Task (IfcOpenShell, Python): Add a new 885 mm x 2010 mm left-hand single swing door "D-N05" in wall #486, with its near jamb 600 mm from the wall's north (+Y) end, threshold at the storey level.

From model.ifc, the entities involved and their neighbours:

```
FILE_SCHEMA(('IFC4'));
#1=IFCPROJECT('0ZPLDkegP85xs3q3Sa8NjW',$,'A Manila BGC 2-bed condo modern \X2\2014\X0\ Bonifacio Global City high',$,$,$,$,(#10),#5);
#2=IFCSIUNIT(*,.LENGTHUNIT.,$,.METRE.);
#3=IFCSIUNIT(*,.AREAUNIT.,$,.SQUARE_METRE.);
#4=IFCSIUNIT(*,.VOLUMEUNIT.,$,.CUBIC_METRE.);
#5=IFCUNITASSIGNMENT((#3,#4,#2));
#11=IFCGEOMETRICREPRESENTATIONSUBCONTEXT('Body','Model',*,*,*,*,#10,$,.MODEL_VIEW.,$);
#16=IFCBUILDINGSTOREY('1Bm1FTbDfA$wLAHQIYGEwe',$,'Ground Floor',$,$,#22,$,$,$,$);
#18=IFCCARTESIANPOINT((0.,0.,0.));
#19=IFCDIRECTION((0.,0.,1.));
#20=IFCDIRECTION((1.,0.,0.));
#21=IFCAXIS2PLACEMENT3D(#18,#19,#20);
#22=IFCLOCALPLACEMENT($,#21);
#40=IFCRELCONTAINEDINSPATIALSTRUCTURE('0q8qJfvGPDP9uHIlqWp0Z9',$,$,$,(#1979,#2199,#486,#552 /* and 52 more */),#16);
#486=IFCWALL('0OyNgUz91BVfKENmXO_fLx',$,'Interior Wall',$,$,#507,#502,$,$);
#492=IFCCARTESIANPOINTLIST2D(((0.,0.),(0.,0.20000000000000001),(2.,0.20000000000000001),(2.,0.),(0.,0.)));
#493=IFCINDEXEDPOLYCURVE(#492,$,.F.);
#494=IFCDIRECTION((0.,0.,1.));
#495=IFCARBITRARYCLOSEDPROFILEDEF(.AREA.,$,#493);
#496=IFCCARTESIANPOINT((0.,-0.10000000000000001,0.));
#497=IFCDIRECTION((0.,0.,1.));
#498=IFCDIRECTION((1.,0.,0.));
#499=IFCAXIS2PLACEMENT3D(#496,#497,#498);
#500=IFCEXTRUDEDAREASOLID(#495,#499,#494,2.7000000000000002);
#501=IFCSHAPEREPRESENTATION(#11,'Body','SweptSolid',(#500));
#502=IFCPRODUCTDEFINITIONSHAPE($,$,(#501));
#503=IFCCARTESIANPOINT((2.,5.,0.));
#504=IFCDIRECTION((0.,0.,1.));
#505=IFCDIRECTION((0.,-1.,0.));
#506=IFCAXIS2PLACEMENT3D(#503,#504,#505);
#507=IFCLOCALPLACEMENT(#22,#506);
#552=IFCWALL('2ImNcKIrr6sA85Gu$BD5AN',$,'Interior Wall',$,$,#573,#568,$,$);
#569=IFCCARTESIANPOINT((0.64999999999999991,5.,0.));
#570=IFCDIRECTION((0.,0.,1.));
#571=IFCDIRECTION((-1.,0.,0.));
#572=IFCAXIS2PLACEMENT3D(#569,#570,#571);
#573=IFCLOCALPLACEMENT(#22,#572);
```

```python
import numpy as np
import ifcopenshell
import ifcopenshell.api.feature
import ifcopenshell.api.geometry
import ifcopenshell.api.root
import ifcopenshell.api.spatial
import ifcopenshell.geom
import ifcopenshell.util.element
import ifcopenshell.util.placement
import ifcopenshell.util.representation
import ifcopenshell.util.shape
import ifcopenshell.util.unit

model = ifcopenshell.open("model.ifc")
unit_scale = ifcopenshell.util.unit.calculate_unit_scale(model)
settings = ifcopenshell.geom.settings()


def volume(element):
    """Net volume in cubic metres, openings subtracted."""
    shape = ifcopenshell.geom.create_shape(settings, element)
    return ifcopenshell.util.shape.get_volume(shape.geometry)


wall = model.by_guid("0OyNgUz91BVfKENmXO_fLx")
storey = ifcopenshell.util.element.get_container(wall, ifc_class="IfcBuildingStorey")
context = ifcopenshell.util.representation.get_context(model, "Model", "Body", "MODEL_VIEW")
before = volume(wall)

width, height, from_end, sill = 0.885, 2.01, 0.6, 0.0  # metres

# The wall runs along its own X axis, and the end named is its -X end.
wall_shape = ifcopenshell.geom.create_shape(settings, wall)
x, y, z = ifcopenshell.util.shape.get_vertices(wall_shape.geometry).T
start = x.min() + from_end
face, thickness = float(y.min()), float(y.max() - y.min())
wall_matrix = ifcopenshell.util.placement.get_local_placement(wall.ObjectPlacement)
level = ifcopenshell.util.placement.get_local_placement(storey.ObjectPlacement)[2, 3]


def in_wall(x, y):
    """Placement at x, y metres in the wall's axes, at sill height."""
    matrix = wall_matrix.copy()
    matrix[:, 3] = wall_matrix @ np.array([x / unit_scale, y / unit_scale, 0.0, 1.0])
    matrix[2, 3] = level + sill / unit_scale
    return matrix


# Opening: a box that overshoots both wall faces by 50 mm.
opening = ifcopenshell.api.root.create_entity(model, ifc_class="IfcOpeningElement", predefined_type="OPENING")
box = ifcopenshell.api.geometry.add_wall_representation(
    model, context=context, length=width, height=height, thickness=thickness + 0.1
)
ifcopenshell.api.geometry.assign_representation(model, product=opening, representation=box)
ifcopenshell.api.geometry.edit_object_placement(model, product=opening, matrix=in_wall(start, face - 0.05), is_si=False)
ifcopenshell.api.feature.add_feature(model, feature=opening, element=wall)

door = ifcopenshell.api.root.create_entity(model, ifc_class="IfcDoor", name="D-N05", predefined_type="DOOR")
door.OverallWidth, door.OverallHeight = width / unit_scale, height / unit_scale
door.OperationType = "SINGLE_SWING_LEFT"
body = ifcopenshell.api.geometry.add_door_representation(
    model,
    context=context,
    overall_width=door.OverallWidth,
    overall_height=door.OverallHeight,
    operation_type="SINGLE_SWING_LEFT",
    lining_properties={"LiningDepth": thickness / unit_scale, "ThresholdDepth": thickness / unit_scale},
)
ifcopenshell.api.geometry.assign_representation(model, product=door, representation=body)
ifcopenshell.api.spatial.assign_container(model, products=[door], relating_structure=storey)
ifcopenshell.api.feature.add_filling(model, opening=opening, element=door)

# The lining spans the wall, so the door starts at the wall face.
ifcopenshell.api.geometry.edit_object_placement(model, product=door, matrix=in_wall(start, face), is_si=False)

after = volume(wall)

print(f"wall volume {before:.3f} -> {after:.3f} m3")

model.write("model_v2.ifc")
```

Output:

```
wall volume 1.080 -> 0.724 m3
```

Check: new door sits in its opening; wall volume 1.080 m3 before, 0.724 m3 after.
